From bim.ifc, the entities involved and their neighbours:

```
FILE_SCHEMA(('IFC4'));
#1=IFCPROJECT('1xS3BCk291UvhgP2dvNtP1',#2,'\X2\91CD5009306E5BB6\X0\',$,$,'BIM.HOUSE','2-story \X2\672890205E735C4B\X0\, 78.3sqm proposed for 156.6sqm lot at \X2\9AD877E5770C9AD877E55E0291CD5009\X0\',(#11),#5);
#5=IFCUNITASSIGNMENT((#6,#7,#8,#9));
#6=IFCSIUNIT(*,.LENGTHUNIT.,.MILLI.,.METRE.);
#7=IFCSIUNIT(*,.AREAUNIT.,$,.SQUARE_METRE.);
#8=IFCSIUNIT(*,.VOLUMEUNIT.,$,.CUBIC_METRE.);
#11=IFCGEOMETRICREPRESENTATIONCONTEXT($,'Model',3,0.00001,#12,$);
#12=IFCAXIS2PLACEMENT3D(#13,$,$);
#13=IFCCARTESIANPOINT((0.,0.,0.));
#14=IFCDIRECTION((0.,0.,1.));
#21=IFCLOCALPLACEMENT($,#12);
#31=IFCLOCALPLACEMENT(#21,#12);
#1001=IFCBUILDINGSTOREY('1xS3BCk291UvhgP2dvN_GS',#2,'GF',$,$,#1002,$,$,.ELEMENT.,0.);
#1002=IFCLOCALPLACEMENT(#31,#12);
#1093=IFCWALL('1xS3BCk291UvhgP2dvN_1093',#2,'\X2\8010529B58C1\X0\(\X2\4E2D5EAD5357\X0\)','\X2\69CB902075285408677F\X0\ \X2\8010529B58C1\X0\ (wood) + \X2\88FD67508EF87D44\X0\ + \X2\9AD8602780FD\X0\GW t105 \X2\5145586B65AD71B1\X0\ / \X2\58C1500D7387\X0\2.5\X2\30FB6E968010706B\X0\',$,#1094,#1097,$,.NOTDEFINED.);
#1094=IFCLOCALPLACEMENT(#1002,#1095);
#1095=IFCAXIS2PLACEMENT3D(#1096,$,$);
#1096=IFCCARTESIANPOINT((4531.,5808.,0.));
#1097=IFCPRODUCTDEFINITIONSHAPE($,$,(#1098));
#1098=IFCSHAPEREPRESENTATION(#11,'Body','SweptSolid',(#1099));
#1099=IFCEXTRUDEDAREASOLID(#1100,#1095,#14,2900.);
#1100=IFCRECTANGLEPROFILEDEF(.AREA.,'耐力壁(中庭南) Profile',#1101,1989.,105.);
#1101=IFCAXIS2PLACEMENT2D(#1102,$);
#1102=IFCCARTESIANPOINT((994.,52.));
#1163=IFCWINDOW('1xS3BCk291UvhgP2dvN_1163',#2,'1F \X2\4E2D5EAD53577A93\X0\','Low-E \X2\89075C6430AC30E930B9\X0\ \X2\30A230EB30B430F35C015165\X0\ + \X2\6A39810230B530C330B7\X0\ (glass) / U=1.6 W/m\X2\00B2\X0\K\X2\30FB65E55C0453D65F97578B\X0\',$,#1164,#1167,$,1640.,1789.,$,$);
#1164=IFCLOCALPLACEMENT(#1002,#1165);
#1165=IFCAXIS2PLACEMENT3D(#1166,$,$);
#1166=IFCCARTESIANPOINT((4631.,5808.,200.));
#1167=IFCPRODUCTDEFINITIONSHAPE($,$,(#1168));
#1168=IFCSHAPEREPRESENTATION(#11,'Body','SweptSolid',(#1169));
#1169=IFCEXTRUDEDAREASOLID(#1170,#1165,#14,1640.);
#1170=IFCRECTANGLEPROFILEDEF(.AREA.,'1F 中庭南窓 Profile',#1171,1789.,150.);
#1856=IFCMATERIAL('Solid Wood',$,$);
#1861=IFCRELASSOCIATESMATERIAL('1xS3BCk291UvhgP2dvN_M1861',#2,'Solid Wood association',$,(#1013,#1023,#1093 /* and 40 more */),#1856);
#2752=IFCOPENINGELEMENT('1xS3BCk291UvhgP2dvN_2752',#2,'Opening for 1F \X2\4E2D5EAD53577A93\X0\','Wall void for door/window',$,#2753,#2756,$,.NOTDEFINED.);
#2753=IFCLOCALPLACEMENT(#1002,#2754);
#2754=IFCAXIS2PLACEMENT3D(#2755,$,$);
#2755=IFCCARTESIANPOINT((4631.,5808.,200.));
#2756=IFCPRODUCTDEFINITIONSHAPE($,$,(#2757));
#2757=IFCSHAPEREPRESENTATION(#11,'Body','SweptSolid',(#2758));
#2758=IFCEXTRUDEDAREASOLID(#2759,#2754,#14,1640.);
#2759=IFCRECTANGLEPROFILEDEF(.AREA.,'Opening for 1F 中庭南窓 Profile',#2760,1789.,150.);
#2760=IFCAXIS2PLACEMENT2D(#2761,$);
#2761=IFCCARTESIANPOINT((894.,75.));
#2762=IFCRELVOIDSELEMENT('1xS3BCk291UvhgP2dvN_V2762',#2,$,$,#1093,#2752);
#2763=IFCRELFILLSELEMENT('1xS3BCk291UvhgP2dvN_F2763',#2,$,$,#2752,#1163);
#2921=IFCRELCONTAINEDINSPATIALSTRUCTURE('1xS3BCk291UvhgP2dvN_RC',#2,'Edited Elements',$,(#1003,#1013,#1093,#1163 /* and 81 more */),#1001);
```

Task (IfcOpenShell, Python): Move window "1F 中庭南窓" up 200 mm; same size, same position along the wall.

```python
import numpy as np
import ifcopenshell
import ifcopenshell.api.geometry
import ifcopenshell.util.placement
import ifcopenshell.util.unit

model = ifcopenshell.open("bim.ifc")
unit_scale = ifcopenshell.util.unit.calculate_unit_scale(model)

window = model.by_guid("1xS3BCk291UvhgP2dvN_1163")
opening = window.FillsVoids[0].RelatingOpeningElement
dz = 0.2 / unit_scale

shift = np.array([0.0, 0.0, dz])
# The window is not placed relative to its opening, so move both.
for product in (opening, window):
    matrix = ifcopenshell.util.placement.get_local_placement(product.ObjectPlacement)
    matrix[:3, 3] += shift
    ifcopenshell.api.geometry.edit_object_placement(model, product=product, matrix=matrix, is_si=False)

print(f"moved by {dz * unit_scale:+.3f} m")

model.write("bim_v2.ifc")
```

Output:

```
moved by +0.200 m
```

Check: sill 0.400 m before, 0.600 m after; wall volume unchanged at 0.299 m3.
